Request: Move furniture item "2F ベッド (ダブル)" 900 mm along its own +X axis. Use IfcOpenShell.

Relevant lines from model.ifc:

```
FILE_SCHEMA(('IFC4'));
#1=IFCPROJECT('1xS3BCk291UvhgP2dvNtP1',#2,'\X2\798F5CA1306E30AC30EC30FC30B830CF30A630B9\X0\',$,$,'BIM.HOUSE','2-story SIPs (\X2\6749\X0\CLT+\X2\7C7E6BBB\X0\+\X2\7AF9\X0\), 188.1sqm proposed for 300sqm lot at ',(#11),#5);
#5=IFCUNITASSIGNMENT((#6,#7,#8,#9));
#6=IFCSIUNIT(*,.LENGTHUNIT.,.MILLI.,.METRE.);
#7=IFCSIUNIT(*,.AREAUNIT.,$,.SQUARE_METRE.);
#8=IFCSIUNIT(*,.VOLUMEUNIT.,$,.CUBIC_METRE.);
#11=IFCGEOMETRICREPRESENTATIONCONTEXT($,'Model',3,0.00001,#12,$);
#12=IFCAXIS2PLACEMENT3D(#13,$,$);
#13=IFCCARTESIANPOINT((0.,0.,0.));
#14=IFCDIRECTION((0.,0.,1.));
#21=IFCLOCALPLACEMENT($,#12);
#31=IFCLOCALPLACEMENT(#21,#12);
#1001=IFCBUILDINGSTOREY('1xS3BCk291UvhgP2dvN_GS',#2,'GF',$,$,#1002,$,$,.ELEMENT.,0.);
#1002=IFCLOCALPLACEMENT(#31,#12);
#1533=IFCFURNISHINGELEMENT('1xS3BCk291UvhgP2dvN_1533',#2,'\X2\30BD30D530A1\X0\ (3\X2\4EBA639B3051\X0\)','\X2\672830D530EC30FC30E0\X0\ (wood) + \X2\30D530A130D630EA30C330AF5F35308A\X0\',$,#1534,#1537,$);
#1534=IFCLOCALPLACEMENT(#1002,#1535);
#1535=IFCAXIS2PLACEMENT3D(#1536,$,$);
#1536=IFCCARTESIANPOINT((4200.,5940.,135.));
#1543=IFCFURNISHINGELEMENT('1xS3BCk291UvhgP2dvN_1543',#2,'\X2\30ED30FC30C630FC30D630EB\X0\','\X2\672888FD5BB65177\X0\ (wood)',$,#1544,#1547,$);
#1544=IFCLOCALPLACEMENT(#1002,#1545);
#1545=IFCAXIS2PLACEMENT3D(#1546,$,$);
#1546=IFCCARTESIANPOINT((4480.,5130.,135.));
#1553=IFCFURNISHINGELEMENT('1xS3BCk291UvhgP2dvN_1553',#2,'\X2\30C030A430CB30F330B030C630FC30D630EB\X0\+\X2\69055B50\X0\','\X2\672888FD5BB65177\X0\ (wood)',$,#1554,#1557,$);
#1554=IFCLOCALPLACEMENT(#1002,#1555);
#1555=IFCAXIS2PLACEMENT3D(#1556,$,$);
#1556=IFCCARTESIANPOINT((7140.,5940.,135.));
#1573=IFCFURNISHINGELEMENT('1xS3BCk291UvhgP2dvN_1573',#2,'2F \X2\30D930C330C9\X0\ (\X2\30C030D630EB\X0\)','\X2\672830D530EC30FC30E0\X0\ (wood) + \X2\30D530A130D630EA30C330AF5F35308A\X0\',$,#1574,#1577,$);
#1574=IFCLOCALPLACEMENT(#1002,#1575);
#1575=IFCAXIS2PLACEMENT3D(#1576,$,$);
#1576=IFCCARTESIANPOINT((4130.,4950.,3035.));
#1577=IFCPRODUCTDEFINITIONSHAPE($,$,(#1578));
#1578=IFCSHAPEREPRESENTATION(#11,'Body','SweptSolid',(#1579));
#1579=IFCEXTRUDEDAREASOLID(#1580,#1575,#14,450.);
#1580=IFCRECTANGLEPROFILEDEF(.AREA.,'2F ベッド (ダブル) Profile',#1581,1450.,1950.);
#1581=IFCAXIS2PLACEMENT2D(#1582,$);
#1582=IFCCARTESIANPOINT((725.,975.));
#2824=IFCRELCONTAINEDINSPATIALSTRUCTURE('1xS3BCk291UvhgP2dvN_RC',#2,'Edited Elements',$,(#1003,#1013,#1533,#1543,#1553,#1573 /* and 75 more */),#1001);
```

```python
import ifcopenshell
import ifcopenshell.api.geometry
import ifcopenshell.util.placement
import ifcopenshell.util.unit

model = ifcopenshell.open("model.ifc")
unit_scale = ifcopenshell.util.unit.calculate_unit_scale(model)

item = model.by_guid("1xS3BCk291UvhgP2dvN_1573")
matrix = ifcopenshell.util.placement.get_local_placement(item.ObjectPlacement)
matrix[:3, 3] += matrix[:3, 0] * 0.9 / unit_scale
ifcopenshell.api.geometry.edit_object_placement(model, product=item, matrix=matrix, is_si=False)

print(ifcopenshell.util.placement.get_local_placement(item.ObjectPlacement).round(3) + 0.0)

model.write("model-out.ifc")
```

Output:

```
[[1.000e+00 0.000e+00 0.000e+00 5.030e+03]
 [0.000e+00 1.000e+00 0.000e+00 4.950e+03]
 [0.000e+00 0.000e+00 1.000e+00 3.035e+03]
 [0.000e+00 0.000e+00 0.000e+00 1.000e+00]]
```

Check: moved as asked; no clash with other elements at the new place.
